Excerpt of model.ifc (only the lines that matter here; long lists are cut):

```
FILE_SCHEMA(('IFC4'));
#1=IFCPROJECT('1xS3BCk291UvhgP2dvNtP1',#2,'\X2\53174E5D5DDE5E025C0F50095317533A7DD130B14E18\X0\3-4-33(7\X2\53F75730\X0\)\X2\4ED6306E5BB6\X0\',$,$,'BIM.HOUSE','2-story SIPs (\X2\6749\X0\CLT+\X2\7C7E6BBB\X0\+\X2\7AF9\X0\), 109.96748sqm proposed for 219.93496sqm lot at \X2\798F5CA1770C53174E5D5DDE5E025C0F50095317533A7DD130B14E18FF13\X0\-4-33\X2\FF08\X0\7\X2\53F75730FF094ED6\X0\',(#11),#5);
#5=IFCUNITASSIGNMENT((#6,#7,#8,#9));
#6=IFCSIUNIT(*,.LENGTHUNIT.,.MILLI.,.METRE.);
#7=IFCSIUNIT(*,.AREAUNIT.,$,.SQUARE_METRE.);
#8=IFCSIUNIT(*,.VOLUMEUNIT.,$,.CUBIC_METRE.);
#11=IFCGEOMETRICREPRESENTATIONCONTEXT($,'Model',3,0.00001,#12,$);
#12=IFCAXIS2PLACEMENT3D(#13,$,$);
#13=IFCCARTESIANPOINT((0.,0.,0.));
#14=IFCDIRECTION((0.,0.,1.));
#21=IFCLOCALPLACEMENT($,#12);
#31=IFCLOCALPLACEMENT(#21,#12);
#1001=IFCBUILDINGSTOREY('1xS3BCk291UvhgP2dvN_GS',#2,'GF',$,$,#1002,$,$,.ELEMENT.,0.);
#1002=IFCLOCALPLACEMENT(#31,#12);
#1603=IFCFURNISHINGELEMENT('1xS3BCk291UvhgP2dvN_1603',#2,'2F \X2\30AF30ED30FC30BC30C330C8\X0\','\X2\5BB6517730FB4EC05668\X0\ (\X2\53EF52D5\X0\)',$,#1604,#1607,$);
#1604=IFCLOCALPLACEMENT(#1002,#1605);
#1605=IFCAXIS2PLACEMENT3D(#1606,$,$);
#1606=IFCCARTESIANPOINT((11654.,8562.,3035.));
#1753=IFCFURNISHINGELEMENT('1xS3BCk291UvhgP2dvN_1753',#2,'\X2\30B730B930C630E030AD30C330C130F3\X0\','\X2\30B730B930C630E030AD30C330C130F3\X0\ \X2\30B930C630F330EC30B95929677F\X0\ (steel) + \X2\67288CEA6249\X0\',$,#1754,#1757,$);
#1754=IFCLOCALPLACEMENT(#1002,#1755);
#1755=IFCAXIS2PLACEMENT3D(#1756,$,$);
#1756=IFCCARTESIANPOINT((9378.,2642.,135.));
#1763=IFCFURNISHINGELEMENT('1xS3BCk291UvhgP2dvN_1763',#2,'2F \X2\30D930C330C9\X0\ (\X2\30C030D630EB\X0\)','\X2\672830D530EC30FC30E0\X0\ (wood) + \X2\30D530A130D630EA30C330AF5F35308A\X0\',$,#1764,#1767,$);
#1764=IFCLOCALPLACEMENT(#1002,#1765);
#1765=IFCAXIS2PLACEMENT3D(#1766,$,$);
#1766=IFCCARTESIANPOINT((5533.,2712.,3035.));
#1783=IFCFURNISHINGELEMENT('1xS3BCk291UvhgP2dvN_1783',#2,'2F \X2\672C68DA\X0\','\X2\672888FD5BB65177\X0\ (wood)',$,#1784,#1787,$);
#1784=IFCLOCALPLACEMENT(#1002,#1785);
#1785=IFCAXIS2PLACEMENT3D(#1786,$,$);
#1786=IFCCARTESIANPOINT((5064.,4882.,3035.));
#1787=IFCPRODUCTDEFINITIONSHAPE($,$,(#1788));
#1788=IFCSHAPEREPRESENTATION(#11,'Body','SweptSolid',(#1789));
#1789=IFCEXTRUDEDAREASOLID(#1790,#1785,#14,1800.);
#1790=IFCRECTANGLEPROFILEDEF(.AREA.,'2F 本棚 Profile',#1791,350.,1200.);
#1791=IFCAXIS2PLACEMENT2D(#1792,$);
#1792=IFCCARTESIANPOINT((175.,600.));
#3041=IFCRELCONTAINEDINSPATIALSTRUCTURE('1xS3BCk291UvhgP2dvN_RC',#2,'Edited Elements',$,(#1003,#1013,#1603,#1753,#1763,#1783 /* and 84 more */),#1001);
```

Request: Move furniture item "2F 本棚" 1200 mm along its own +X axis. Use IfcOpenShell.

```python
import ifcopenshell
import ifcopenshell.api.geometry
import ifcopenshell.util.placement
import ifcopenshell.util.unit

model = ifcopenshell.open("model.ifc")
unit_scale = ifcopenshell.util.unit.calculate_unit_scale(model)

item = model.by_id(1783)
matrix = ifcopenshell.util.placement.get_local_placement(item.ObjectPlacement)
matrix[:3, 3] += matrix[:3, 0] * 1.2 / unit_scale
ifcopenshell.api.geometry.edit_object_placement(model, product=item, matrix=matrix, is_si=False)

print(ifcopenshell.util.placement.get_local_placement(item.ObjectPlacement).round(3) + 0.0)

model.write("model_updated.ifc")
```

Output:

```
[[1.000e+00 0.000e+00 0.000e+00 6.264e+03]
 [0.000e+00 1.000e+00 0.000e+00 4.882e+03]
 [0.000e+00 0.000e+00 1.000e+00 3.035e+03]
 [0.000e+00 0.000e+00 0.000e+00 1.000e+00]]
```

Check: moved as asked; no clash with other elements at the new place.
